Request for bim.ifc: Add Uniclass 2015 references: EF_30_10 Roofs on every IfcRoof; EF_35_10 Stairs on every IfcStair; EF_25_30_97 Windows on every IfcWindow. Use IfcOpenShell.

First a look at what the model holds.

```python
import ifcopenshell

model = ifcopenshell.open("bim.ifc")
print(model.schema)
print("classifications:", [c.Name for c in model.by_type("IfcClassification")])
for ifc_class in ("IfcDoor", "IfcRoof", "IfcStair", "IfcWall", "IfcWindow"):
    print(ifc_class, len(model.by_type(ifc_class)))
```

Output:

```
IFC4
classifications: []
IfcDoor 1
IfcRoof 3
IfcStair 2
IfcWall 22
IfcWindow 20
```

```python
import ifcopenshell
import ifcopenshell.api.classification

model = ifcopenshell.open("bim.ifc")

system = ifcopenshell.api.classification.add_classification(model, classification="Uniclass 2015")

codes = {
    "IfcRoof": ("EF_30_10", "Roofs"),
    "IfcStair": ("EF_35_10", "Stairs"),
    "IfcWindow": ("EF_25_30_97", "Windows"),
}
for ifc_class, (code, name) in codes.items():
    products = model.by_type(ifc_class)
    ifcopenshell.api.classification.add_reference(
        model, products=products, classification=system, identification=code, name=name
    )
    print(code, len(products))

model.write("bim_updated.ifc")
```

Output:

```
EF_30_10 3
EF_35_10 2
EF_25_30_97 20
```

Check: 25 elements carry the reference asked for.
